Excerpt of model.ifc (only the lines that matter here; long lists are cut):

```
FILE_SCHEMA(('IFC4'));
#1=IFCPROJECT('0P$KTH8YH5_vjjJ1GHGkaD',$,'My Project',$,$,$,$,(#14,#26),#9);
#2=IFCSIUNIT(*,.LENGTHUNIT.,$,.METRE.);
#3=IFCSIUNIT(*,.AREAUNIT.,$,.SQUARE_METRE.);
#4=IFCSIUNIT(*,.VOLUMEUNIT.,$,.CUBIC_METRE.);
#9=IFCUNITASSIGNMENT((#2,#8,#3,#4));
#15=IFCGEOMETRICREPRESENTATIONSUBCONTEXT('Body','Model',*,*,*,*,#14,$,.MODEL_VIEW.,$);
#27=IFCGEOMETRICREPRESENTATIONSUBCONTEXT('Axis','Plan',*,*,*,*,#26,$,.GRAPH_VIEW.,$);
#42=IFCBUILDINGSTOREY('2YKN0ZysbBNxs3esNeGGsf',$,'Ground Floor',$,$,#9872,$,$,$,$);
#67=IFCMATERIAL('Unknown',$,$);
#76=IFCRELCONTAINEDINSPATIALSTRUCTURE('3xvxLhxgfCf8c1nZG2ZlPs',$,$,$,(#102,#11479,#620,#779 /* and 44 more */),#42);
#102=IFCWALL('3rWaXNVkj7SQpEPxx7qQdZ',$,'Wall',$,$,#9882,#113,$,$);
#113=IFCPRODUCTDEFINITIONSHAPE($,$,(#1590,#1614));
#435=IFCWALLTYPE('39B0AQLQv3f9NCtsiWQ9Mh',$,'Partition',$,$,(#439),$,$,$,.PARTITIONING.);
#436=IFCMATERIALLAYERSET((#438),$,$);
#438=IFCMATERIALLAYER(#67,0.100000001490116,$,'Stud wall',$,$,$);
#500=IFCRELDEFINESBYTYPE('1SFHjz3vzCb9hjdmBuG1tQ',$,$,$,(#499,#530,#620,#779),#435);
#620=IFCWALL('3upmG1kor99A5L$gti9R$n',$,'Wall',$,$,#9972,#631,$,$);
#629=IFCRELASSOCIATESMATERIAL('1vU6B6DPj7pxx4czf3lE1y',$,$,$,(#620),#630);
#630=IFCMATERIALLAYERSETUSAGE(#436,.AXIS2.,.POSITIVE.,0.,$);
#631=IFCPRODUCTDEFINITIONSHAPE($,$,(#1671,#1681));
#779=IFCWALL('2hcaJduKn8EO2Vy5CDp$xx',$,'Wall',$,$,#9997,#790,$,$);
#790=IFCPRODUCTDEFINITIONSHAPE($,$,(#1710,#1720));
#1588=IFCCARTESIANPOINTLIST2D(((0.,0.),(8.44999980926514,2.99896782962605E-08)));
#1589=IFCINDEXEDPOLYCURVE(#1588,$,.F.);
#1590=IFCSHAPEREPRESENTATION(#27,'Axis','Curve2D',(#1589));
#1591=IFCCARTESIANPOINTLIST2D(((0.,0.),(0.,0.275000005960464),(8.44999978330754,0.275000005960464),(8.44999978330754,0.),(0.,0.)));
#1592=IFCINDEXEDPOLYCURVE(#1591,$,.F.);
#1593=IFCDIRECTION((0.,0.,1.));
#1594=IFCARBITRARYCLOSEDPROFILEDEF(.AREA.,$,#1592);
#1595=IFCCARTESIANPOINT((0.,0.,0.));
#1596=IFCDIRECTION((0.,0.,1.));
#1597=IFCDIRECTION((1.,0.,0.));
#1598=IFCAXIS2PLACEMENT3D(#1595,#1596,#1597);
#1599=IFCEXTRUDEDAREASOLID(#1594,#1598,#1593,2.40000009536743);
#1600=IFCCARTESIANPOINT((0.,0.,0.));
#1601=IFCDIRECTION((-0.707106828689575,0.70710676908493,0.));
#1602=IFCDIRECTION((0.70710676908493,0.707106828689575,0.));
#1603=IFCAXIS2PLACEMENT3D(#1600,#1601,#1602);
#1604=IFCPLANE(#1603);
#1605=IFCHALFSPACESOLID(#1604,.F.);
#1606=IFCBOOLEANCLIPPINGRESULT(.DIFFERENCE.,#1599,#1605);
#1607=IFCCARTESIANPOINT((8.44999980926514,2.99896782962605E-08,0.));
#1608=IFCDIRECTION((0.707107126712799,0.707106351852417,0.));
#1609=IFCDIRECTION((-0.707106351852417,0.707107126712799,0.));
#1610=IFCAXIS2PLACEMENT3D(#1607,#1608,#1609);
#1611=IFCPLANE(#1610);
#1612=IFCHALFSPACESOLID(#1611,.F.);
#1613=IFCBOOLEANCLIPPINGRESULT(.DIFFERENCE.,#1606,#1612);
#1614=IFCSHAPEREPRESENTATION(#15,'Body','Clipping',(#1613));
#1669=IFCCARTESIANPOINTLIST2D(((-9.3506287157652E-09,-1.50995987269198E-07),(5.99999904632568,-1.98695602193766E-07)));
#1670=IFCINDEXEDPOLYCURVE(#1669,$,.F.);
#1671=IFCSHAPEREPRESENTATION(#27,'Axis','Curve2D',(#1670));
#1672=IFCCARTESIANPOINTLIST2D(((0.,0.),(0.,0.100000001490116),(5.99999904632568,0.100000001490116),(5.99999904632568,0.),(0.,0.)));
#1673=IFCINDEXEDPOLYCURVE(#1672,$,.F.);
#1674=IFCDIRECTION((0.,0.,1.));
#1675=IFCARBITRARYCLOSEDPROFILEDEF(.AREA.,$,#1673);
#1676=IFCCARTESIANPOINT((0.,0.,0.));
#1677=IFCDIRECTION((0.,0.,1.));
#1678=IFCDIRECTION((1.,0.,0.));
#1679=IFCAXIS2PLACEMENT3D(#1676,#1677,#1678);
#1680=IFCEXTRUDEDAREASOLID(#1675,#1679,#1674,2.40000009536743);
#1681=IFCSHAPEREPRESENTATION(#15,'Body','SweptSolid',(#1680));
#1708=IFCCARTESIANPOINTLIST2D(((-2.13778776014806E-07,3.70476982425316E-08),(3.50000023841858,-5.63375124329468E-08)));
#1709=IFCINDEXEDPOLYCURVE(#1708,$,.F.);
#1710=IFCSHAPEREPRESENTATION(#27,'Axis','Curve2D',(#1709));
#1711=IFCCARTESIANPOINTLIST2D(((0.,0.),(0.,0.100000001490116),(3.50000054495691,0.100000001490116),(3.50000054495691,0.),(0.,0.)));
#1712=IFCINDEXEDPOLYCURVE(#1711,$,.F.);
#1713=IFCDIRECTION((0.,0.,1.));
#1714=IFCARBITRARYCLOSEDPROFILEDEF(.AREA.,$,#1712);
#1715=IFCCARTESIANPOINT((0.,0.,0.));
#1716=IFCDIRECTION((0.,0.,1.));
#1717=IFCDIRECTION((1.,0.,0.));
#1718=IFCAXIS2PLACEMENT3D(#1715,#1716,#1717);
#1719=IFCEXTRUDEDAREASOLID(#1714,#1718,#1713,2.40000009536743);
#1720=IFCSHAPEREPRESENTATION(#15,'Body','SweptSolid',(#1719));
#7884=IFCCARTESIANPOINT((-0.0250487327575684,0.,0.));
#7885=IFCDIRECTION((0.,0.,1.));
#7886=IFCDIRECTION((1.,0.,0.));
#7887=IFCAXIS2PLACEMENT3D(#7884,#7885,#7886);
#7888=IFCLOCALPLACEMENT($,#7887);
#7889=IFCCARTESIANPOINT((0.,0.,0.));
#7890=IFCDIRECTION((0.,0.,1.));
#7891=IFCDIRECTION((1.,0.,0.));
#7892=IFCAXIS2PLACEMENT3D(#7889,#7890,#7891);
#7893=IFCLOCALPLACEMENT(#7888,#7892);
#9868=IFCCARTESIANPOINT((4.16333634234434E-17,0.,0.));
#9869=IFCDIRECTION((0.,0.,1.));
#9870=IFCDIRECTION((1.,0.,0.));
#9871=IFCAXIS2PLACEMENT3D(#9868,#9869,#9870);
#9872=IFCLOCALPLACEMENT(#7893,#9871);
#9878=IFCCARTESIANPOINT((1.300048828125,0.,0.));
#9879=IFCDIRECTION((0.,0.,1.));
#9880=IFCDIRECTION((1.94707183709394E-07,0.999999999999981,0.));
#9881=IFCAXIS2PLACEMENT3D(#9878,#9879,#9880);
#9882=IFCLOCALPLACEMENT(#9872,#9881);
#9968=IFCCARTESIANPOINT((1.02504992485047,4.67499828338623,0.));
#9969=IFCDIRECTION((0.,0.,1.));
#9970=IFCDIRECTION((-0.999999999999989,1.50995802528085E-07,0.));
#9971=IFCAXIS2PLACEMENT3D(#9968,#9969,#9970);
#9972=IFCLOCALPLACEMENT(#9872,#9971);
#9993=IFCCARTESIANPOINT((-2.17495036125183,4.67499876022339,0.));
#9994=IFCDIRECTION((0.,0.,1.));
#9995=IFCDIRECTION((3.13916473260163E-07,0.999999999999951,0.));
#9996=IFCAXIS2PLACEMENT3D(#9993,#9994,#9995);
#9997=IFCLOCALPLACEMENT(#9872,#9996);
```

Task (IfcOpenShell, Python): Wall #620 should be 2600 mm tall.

```python
import ifcopenshell
import ifcopenshell.geom
import ifcopenshell.util.representation
import ifcopenshell.util.shape

model = ifcopenshell.open("model.ifc")
settings = ifcopenshell.geom.settings()


def volume(element):
    """Net volume in cubic metres, openings subtracted."""
    shape = ifcopenshell.geom.create_shape(settings, element)
    return ifcopenshell.util.shape.get_volume(shape.geometry)


wall = model.by_guid("3upmG1kor99A5L$gti9R$n")
before = volume(wall)

body = ifcopenshell.util.representation.get_representation(wall, "Model", "Body")
solid = body.Items[0]
old_height = solid.Depth
solid.Depth = 2.6
after = volume(wall)

print(f"height {old_height:g} -> {solid.Depth:g}, volume {before:.3f} -> {after:.3f} m3")

model.write("model_updated.ifc")
```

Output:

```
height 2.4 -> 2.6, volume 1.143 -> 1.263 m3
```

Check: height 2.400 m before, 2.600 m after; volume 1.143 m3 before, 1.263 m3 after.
